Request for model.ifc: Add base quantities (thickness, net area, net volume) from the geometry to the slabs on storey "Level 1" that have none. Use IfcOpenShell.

First a look at what the model holds.

```python
import ifcopenshell
import ifcopenshell.util.element
import ifcopenshell.util.unit

model = ifcopenshell.open("model.ifc")
print(model.schema)
for unit_type in ("LENGTHUNIT", "AREAUNIT", "VOLUMEUNIT"):
    print(unit_type, ifcopenshell.util.unit.calculate_unit_scale(model, unit_type))
storey = next(s for s in model.by_type("IfcBuildingStorey") if s.Name == "Level 1")
slabs = [e for e in ifcopenshell.util.element.get_decomposition(storey) if e.is_a("IfcSlab")]
for e in sorted(slabs, key=lambda e: e.id()):
    print(e.id(), e.is_a(), e.Name, list(ifcopenshell.util.element.get_psets(e, qtos_only=True)), sep=" | ")
```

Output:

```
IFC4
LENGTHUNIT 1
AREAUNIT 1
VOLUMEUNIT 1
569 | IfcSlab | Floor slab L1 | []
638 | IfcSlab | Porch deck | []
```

```python
import ifcopenshell
import ifcopenshell.api.pset
import ifcopenshell.geom
import ifcopenshell.util.element
import ifcopenshell.util.shape
import ifcopenshell.util.unit

model = ifcopenshell.open("model.ifc")
unit_scale = ifcopenshell.util.unit.calculate_unit_scale(model)
area_scale = ifcopenshell.util.unit.calculate_unit_scale(model, "AREAUNIT")
volume_scale = ifcopenshell.util.unit.calculate_unit_scale(model, "VOLUMEUNIT")
settings = ifcopenshell.geom.settings()

storey = next(s for s in model.by_type("IfcBuildingStorey") if s.Name == "Level 1")
slabs = [e for e in ifcopenshell.util.element.get_decomposition(storey) if e.is_a("IfcSlab")]

for e in sorted(slabs, key=lambda e: e.id()):
    if ifcopenshell.util.element.get_psets(e, qtos_only=True, should_inherit=False):
        continue
    # Geometry comes back in metres, in the element's own axes.
    shape = ifcopenshell.geom.create_shape(settings, e)
    values = {
        "Width": ifcopenshell.util.shape.get_z(shape.geometry) / unit_scale,
        "NetArea": ifcopenshell.util.shape.get_footprint_area(shape.geometry) / area_scale,
        "NetVolume": ifcopenshell.util.shape.get_volume(shape.geometry) / volume_scale,
    }
    qto = ifcopenshell.api.pset.add_qto(model, product=e, name="Qto_SlabBaseQuantities")
    ifcopenshell.api.pset.edit_qto(model, qto=qto, properties=values)
    print(e.id(), {k: round(v, 3) for k, v in values.items()})

model.write("model_rev.ifc")
```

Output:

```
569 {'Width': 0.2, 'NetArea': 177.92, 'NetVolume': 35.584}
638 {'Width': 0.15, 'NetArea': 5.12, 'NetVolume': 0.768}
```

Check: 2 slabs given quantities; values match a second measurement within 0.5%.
